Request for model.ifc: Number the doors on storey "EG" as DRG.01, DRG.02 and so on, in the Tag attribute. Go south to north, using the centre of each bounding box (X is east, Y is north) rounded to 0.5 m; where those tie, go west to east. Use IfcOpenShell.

First a look at what the model holds.

```python
import ifcopenshell
import ifcopenshell.util.element
import ifcopenshell.util.placement

model = ifcopenshell.open("model.ifc")
print(model.schema)
storey = next(s for s in model.by_type("IfcBuildingStorey") if s.Name == "EG")
doors = [e for e in ifcopenshell.util.element.get_decomposition(storey) if e.is_a("IfcDoor")]
for e in sorted(doors, key=lambda e: e.id()):
    origin = ifcopenshell.util.placement.get_local_placement(e.ObjectPlacement)[:3, 3]
    print(e.id(), e.Tag, e.Name, origin.round(2) + 0.0, sep=" | ")
```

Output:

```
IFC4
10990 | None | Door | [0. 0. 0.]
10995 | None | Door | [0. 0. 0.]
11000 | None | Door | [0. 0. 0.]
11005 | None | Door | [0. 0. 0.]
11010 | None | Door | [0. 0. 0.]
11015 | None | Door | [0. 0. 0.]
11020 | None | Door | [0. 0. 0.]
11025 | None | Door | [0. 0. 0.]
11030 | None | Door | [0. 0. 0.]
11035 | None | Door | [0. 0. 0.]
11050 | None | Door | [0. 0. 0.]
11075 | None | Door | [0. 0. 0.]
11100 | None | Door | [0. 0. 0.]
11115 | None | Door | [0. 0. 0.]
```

```python
import ifcopenshell
import ifcopenshell.geom
import ifcopenshell.util.element
import ifcopenshell.util.shape

model = ifcopenshell.open("model.ifc")
settings = ifcopenshell.geom.settings()
settings.set("use-world-coords", True)


def centre(element):
    shape = ifcopenshell.geom.create_shape(settings, element)
    return ifcopenshell.util.shape.get_bbox_centroid(shape.geometry)


storey = next(s for s in model.by_type("IfcBuildingStorey") if s.Name == "EG")
doors = [e for e in ifcopenshell.util.element.get_decomposition(storey) if e.is_a("IfcDoor")]

# Insertion points can sit at a corner or the storey origin, so sort by the geometry (in metres).
centres = {e: centre(e) for e in doors}
doors.sort(key=lambda e: (round(centres[e][1] / 0.5), centres[e][0]))

for i, e in enumerate(doors, start=1):
    number = f"DRG.{i:02d}"
    e.Tag = number
    print(e.id(), number)

model.write("model_edited.ifc")
```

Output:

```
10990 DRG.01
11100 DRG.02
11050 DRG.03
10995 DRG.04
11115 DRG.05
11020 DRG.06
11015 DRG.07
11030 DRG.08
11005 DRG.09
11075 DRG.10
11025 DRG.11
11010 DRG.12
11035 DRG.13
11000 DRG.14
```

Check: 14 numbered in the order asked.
